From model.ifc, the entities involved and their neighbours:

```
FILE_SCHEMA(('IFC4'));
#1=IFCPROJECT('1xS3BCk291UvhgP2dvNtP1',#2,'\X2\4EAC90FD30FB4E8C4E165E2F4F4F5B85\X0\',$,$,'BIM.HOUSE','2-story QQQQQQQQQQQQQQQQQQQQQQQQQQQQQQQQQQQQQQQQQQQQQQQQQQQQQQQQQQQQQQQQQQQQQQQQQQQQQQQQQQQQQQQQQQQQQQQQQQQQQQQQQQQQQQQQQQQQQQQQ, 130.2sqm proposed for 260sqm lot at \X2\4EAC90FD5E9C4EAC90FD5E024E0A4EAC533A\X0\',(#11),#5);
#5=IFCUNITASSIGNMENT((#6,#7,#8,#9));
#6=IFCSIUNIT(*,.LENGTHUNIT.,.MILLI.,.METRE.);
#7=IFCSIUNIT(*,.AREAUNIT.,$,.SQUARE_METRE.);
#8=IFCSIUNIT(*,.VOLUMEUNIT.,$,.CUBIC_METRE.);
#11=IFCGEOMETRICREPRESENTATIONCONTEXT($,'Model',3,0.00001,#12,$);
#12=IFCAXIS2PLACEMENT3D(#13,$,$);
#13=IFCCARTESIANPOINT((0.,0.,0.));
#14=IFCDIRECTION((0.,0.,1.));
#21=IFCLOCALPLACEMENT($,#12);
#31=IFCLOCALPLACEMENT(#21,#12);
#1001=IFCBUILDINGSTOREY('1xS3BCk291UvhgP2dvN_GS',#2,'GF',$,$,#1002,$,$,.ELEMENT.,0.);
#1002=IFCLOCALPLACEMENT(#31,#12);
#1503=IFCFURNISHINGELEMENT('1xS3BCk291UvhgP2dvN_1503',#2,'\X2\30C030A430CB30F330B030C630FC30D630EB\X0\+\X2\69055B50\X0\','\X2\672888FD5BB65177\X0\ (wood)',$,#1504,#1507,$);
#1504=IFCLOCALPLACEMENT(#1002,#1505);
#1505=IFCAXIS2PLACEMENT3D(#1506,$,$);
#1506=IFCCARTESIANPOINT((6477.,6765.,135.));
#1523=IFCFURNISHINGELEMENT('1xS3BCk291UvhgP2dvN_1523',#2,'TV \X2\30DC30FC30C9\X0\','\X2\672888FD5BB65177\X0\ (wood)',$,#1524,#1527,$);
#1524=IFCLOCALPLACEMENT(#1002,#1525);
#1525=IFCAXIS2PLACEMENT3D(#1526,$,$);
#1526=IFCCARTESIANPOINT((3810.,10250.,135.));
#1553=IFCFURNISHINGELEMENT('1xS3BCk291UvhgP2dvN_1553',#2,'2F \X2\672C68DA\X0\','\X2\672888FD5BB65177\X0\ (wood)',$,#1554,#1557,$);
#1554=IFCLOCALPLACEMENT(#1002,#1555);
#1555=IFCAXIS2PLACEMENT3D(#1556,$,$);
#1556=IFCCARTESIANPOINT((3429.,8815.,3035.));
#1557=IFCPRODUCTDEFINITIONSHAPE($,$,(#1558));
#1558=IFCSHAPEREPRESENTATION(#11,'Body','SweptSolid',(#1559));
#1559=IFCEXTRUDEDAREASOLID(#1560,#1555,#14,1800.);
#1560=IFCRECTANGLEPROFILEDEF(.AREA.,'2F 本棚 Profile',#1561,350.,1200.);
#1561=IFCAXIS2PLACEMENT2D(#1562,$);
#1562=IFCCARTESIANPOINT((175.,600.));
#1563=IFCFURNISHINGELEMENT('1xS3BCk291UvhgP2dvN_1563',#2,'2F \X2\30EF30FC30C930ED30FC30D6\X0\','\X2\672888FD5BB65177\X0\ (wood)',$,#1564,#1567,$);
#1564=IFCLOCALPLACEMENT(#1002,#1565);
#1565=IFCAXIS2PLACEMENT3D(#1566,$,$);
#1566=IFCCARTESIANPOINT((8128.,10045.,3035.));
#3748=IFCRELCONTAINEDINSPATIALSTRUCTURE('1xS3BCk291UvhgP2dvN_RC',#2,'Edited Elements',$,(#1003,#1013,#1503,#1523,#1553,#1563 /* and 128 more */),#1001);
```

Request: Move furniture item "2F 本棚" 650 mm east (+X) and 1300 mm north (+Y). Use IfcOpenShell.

```python
import ifcopenshell
import ifcopenshell.api.geometry
import ifcopenshell.util.placement
import ifcopenshell.util.unit

model = ifcopenshell.open("model.ifc")
unit_scale = ifcopenshell.util.unit.calculate_unit_scale(model)

item = model.by_guid("1xS3BCk291UvhgP2dvN_1553")
matrix = ifcopenshell.util.placement.get_local_placement(item.ObjectPlacement)
matrix[0, 3] += 0.65 / unit_scale
matrix[1, 3] += 1.3 / unit_scale
ifcopenshell.api.geometry.edit_object_placement(model, product=item, matrix=matrix, is_si=False)

print(ifcopenshell.util.placement.get_local_placement(item.ObjectPlacement).round(3) + 0.0)

model.write("model_rev.ifc")
```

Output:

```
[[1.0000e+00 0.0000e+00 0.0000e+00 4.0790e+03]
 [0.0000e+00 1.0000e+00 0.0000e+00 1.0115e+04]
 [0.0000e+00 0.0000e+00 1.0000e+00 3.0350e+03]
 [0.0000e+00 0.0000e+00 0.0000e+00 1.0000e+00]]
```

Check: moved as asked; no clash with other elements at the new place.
